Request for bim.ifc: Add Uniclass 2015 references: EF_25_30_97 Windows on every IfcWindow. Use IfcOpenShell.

First a look at what the model holds.

```python
import ifcopenshell

model = ifcopenshell.open("bim.ifc")
print(model.schema)
print("classifications:", [c.Name for c in model.by_type("IfcClassification")])
for ifc_class in ("IfcDoor", "IfcRoof", "IfcStair", "IfcWall", "IfcWindow"):
    print(ifc_class, len(model.by_type(ifc_class)))
```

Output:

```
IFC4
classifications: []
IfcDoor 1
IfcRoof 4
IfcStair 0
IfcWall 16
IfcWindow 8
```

```python
import ifcopenshell
import ifcopenshell.api.classification

model = ifcopenshell.open("bim.ifc")

system = ifcopenshell.api.classification.add_classification(model, classification="Uniclass 2015")

codes = {
    "IfcWindow": ("EF_25_30_97", "Windows"),
}
for ifc_class, (code, name) in codes.items():
    products = model.by_type(ifc_class)
    ifcopenshell.api.classification.add_reference(
        model, products=products, classification=system, identification=code, name=name
    )
    print(code, len(products))

model.write("bim_updated.ifc")
```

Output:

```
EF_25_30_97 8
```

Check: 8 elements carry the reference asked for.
